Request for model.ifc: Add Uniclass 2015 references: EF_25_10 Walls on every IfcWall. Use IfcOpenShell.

First a look at what the model holds.

```python
import ifcopenshell

model = ifcopenshell.open("model.ifc")
print(model.schema)
print("classifications:", [c.Name for c in model.by_type("IfcClassification")])
for ifc_class in ("IfcDoor", "IfcRoof", "IfcStair", "IfcWall", "IfcWindow"):
    print(ifc_class, len(model.by_type(ifc_class)))
```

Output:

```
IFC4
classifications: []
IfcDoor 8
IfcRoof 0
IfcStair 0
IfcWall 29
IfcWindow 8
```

```python
import ifcopenshell
import ifcopenshell.api.classification

model = ifcopenshell.open("model.ifc")

system = ifcopenshell.api.classification.add_classification(model, classification="Uniclass 2015")

codes = {
    "IfcWall": ("EF_25_10", "Walls"),
}
for ifc_class, (code, name) in codes.items():
    products = model.by_type(ifc_class)
    ifcopenshell.api.classification.add_reference(
        model, products=products, classification=system, identification=code, name=name
    )
    print(code, len(products))

model.write("model_rev.ifc")
```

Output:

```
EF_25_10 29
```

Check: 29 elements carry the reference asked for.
